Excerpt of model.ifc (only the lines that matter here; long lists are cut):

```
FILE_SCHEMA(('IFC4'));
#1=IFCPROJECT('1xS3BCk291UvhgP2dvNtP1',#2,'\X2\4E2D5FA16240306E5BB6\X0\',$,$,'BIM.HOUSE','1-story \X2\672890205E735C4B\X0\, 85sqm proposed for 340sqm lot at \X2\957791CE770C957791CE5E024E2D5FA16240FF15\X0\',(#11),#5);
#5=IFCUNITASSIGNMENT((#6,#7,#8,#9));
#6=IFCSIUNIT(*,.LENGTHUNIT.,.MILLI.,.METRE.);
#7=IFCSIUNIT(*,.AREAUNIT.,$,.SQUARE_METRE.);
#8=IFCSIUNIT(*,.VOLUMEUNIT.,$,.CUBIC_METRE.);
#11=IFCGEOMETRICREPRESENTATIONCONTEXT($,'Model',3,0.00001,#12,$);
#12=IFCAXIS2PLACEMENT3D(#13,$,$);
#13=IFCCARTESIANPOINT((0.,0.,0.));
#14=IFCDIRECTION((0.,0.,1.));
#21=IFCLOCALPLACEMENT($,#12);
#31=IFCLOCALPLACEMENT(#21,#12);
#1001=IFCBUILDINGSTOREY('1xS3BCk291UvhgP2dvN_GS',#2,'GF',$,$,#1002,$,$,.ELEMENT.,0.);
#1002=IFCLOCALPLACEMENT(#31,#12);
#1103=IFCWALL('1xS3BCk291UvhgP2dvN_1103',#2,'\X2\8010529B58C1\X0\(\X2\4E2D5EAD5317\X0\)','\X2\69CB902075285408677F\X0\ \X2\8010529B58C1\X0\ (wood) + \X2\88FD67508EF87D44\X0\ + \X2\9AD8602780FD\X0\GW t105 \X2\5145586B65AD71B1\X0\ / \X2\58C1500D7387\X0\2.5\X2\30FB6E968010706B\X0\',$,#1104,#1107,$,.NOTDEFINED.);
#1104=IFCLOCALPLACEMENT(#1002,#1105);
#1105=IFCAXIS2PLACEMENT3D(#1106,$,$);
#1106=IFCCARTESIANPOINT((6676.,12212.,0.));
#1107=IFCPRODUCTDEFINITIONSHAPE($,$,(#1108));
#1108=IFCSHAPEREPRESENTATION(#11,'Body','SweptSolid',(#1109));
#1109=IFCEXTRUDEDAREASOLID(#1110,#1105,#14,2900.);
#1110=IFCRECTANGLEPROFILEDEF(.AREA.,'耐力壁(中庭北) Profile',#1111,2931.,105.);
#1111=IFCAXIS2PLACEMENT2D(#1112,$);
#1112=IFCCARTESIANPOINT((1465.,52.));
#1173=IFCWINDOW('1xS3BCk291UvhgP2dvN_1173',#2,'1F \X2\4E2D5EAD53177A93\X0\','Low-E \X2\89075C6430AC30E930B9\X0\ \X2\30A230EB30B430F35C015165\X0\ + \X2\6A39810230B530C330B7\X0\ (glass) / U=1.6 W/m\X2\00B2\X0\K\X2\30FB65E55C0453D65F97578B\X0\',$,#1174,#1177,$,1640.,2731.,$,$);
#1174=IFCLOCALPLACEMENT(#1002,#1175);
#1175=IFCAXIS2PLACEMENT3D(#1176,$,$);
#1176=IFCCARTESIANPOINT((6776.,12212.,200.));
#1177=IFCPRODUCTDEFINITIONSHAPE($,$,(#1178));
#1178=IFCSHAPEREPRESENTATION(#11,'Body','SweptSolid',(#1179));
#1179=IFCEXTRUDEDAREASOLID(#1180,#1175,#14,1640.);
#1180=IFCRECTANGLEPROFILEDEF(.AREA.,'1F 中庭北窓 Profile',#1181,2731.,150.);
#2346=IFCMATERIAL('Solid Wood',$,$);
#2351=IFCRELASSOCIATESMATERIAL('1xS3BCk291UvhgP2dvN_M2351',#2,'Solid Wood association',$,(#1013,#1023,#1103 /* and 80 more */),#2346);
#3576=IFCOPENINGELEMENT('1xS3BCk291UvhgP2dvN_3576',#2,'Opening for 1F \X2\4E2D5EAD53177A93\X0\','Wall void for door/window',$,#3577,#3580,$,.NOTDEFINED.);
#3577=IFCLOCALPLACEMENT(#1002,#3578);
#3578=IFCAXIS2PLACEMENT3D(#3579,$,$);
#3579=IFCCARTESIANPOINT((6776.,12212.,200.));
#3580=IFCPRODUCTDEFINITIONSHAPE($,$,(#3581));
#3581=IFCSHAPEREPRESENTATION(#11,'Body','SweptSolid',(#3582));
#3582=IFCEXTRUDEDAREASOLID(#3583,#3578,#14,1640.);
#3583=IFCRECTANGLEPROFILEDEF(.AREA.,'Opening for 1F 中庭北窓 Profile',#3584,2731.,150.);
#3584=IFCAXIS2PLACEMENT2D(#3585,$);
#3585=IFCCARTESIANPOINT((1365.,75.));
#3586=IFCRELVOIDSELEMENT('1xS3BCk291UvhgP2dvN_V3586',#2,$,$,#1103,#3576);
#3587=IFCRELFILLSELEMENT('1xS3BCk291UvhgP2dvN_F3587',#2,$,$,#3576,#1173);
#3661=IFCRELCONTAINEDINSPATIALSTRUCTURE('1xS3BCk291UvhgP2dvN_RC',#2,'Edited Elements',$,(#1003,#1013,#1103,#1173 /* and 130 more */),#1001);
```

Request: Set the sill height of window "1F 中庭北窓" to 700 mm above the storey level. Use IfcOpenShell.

```python
import numpy as np
import ifcopenshell
import ifcopenshell.api.geometry
import ifcopenshell.geom
import ifcopenshell.util.element
import ifcopenshell.util.placement
import ifcopenshell.util.shape
import ifcopenshell.util.unit

model = ifcopenshell.open("model.ifc")
unit_scale = ifcopenshell.util.unit.calculate_unit_scale(model)

window = model.by_guid("1xS3BCk291UvhgP2dvN_1173")
opening = window.FillsVoids[0].RelatingOpeningElement
storey = ifcopenshell.util.element.get_container(window, ifc_class="IfcBuildingStorey")
level = ifcopenshell.util.placement.get_local_placement(storey.ObjectPlacement)[2, 3]

# The opening's origin need not be at the sill, so measure its lowest point.
shape = ifcopenshell.geom.create_shape(ifcopenshell.geom.settings(), opening)
bottom = ifcopenshell.util.shape.get_shape_bottom_elevation(shape, shape.geometry) / unit_scale
dz = level + 0.7 / unit_scale - bottom

shift = np.array([0.0, 0.0, dz])
# The window is not placed relative to its opening, so move both.
for product in (opening, window):
    matrix = ifcopenshell.util.placement.get_local_placement(product.ObjectPlacement)
    matrix[:3, 3] += shift
    ifcopenshell.api.geometry.edit_object_placement(model, product=product, matrix=matrix, is_si=False)

print(f"moved by {dz * unit_scale:+.3f} m")

model.write("model-out.ifc")
```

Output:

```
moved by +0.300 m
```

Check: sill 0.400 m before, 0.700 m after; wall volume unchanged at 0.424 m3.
